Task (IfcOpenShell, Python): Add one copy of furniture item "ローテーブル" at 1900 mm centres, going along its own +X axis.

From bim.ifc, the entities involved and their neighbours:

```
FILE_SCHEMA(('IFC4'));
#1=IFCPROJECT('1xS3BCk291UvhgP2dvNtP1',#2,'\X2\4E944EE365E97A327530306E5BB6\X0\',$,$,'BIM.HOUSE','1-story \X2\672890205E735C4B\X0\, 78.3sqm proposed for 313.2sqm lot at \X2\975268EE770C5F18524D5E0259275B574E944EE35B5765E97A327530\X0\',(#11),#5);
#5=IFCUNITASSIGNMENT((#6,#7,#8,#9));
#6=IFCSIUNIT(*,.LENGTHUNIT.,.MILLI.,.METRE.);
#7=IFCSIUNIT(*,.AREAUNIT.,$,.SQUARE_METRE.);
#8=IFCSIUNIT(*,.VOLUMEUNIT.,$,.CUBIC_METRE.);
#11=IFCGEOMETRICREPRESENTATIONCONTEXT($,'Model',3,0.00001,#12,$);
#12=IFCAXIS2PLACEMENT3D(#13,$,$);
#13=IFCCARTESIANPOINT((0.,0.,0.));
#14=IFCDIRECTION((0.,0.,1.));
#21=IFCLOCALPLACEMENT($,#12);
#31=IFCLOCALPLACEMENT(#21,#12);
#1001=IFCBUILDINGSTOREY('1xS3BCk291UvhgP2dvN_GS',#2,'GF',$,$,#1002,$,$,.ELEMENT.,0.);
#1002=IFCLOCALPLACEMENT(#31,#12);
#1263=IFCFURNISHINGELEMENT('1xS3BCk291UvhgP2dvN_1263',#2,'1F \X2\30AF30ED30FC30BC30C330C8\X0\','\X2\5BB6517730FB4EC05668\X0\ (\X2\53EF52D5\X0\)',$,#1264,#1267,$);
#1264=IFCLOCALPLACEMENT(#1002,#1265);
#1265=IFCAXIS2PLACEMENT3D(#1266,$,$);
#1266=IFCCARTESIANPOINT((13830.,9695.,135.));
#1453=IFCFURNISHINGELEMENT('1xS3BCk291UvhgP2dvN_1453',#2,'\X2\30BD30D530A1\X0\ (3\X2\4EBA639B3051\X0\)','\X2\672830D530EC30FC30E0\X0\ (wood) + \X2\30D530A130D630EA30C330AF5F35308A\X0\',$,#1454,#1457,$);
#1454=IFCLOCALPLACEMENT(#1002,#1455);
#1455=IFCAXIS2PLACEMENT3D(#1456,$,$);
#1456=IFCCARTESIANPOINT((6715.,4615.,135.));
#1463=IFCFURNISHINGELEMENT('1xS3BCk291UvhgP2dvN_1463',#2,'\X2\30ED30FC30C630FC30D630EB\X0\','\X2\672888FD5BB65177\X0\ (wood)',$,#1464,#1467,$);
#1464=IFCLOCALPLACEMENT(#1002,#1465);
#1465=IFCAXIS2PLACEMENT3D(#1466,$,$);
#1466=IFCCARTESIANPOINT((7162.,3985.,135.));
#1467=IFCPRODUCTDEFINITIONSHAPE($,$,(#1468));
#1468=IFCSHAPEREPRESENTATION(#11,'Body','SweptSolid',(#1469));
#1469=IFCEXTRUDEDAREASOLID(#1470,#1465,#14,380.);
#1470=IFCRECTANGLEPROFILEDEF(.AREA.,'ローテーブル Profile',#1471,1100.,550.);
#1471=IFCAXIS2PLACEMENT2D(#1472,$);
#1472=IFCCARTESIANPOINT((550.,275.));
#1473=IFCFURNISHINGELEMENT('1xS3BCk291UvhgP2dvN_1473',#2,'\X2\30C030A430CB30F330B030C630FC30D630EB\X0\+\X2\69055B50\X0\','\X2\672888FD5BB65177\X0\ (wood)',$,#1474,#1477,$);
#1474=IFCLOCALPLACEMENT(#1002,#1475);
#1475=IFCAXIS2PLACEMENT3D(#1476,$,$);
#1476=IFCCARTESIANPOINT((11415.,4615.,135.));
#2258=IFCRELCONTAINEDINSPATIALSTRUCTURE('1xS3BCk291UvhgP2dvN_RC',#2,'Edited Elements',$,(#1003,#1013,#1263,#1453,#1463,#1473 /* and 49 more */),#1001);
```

```python
import ifcopenshell
import ifcopenshell.api.geometry
import ifcopenshell.api.root
import ifcopenshell.util.element
import ifcopenshell.util.placement

model = ifcopenshell.open("bim.ifc")


def reuse_history(source, copy):
    """copy_class also copies each property set's owner history, people and application; keep the originals."""
    for rel in copy.IsDefinedBy:
        if rel.is_a("IfcRelDefinesByProperties") and (history := rel.RelatingPropertyDefinition.OwnerHistory):
            rel.RelatingPropertyDefinition.OwnerHistory = source.OwnerHistory
            ifcopenshell.util.element.remove_deep2(model, history)


source = model.by_guid("1xS3BCk291UvhgP2dvN_1463")
base = ifcopenshell.util.placement.get_local_placement(source.ObjectPlacement)
step = base[:3, 0] * 1900.0

for i in range(1, 2):
    copy = ifcopenshell.api.root.copy_class(model, product=source)
    copy.Representation = ifcopenshell.util.element.copy_deep(
        model, source.Representation, exclude=["IfcGeometricRepresentationContext", "IfcRepresentationMap"]
    )
    reuse_history(source, copy)
    matrix = base.copy()
    matrix[:3, 3] += i * step
    print("added at", matrix[:3, 3].round(3) + 0.0)
    ifcopenshell.api.geometry.edit_object_placement(model, product=copy, matrix=matrix, is_si=False)

model.write("bim-out.ifc")
```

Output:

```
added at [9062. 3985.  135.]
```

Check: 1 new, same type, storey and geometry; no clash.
